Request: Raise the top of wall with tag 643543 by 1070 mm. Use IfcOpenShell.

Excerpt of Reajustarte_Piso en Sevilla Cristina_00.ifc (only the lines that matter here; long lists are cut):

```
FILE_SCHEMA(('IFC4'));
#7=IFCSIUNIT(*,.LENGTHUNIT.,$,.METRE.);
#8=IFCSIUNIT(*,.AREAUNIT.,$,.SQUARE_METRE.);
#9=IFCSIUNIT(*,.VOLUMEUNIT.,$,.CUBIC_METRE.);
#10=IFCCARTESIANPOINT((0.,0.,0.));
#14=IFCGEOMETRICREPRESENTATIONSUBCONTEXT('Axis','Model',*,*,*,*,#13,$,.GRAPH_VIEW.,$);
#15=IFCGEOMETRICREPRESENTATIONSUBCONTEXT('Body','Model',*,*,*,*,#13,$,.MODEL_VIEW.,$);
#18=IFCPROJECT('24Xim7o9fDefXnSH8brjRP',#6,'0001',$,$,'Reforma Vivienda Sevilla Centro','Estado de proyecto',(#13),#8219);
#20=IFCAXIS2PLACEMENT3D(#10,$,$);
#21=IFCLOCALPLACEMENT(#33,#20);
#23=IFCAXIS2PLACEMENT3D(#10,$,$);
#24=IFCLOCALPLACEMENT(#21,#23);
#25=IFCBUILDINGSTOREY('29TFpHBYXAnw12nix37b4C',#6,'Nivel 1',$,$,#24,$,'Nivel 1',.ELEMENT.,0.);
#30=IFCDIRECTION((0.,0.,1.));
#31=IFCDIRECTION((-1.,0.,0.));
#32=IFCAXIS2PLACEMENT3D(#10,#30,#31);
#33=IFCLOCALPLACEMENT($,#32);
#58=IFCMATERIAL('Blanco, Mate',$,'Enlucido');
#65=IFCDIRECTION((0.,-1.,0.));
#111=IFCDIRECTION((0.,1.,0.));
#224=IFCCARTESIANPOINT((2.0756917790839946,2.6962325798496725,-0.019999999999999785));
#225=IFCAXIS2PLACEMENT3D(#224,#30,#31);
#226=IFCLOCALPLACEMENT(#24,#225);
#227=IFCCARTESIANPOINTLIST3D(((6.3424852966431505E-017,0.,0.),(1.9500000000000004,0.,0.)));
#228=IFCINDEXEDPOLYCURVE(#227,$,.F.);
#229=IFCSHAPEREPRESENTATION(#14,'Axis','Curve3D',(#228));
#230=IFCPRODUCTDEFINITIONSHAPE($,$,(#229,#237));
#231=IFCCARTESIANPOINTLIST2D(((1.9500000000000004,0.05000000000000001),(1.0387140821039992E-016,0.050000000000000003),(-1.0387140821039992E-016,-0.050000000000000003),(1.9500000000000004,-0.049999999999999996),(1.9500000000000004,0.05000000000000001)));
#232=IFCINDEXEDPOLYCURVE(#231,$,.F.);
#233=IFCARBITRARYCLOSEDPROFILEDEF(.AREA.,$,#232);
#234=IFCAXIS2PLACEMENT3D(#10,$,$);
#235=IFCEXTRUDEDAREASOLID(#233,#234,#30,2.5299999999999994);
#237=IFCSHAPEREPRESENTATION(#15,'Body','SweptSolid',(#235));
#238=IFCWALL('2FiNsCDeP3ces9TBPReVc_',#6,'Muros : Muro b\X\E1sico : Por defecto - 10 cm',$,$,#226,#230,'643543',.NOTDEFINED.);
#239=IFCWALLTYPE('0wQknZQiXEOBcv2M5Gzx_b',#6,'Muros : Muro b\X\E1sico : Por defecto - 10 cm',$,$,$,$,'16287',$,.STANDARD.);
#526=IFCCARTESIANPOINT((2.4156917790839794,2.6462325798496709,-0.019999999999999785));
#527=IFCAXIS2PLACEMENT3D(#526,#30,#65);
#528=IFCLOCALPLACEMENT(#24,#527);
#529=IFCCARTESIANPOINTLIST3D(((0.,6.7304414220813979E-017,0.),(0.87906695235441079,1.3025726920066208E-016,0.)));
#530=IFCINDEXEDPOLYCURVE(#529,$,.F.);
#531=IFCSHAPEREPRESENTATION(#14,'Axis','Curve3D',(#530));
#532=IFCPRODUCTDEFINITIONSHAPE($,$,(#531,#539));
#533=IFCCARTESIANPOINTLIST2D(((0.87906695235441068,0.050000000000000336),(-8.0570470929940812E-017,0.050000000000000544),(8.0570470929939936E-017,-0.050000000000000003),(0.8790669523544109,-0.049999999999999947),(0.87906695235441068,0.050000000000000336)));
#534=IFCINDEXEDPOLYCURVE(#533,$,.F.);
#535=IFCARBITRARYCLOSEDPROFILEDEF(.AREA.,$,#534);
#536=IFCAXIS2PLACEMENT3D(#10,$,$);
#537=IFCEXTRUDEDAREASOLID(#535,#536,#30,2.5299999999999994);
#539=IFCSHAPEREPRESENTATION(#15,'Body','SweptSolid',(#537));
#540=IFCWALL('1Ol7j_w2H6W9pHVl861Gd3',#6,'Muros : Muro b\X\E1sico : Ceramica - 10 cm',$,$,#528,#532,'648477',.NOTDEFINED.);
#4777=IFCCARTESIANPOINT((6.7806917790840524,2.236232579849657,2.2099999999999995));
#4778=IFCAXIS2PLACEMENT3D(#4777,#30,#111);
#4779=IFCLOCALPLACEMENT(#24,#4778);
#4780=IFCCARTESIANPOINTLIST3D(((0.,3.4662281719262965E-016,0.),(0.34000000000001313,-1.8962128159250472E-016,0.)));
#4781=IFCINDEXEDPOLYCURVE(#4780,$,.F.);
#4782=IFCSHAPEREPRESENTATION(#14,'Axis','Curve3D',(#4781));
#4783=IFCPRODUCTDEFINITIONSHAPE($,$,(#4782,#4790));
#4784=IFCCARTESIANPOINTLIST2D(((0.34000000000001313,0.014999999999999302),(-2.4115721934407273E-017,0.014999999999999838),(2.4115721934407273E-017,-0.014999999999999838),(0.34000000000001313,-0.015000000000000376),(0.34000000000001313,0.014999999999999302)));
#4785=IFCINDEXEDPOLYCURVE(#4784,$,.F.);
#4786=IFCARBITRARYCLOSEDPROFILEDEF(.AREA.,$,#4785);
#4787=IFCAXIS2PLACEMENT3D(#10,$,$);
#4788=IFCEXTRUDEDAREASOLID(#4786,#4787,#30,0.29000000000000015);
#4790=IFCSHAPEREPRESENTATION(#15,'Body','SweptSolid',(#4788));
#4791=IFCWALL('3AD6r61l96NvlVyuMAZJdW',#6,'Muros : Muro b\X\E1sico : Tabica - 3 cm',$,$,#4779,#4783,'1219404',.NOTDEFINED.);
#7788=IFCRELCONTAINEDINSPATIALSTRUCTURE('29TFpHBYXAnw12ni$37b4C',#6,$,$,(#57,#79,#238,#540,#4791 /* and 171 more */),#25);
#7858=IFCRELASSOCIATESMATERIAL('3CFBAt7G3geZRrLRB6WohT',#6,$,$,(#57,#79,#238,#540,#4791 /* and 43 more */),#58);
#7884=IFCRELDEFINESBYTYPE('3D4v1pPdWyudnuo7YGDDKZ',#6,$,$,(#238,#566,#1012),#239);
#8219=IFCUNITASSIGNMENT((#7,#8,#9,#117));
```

```python
import ifcopenshell
import ifcopenshell.geom
import ifcopenshell.util.representation
import ifcopenshell.util.shape

model = ifcopenshell.open("Reajustarte_Piso en Sevilla Cristina_00.ifc")
settings = ifcopenshell.geom.settings()


def volume(element):
    """Net volume in cubic metres, openings subtracted."""
    shape = ifcopenshell.geom.create_shape(settings, element)
    return ifcopenshell.util.shape.get_volume(shape.geometry)


wall = model.by_id(238)
before = volume(wall)

body = ifcopenshell.util.representation.get_representation(wall, "Model", "Body")
solid = body.Items[0]
old_height = solid.Depth
solid.Depth += 1.07
after = volume(wall)

print(f"height {old_height:g} -> {solid.Depth:g}, volume {before:.3f} -> {after:.3f} m3")

model.write("Reajustarte_Piso en Sevilla Cristina_00-out.ifc")
```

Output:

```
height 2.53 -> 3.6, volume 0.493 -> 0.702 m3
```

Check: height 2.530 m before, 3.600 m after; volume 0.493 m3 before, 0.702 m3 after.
